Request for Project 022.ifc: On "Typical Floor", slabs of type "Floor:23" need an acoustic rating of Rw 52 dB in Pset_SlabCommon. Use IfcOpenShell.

First a look at what the model holds.

```python
import ifcopenshell
import ifcopenshell.util.element

model = ifcopenshell.open("Project 022.ifc")
print(model.schema)
storey = next(s for s in model.by_type("IfcBuildingStorey") if s.Name == "Typical Floor")
slabs = [e for e in ifcopenshell.util.element.get_decomposition(storey) if e.is_a("IfcSlab")]
seen = {}
for e in slabs:
    element_type = ifcopenshell.util.element.get_type(e)
    key = (element_type.Name if element_type != e and element_type else None, ifcopenshell.util.element.get_pset(e, "Pset_SlabCommon", "AcousticRating"))
    seen[key] = seen.get(key, 0) + 1
for (name, value), count in sorted(seen.items(), key=str):
    print(count, "x", name, "|", value)
```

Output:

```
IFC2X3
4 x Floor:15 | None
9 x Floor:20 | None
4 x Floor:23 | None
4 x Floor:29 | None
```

```python
import ifcopenshell
import ifcopenshell.api.pset
import ifcopenshell.util.element

model = ifcopenshell.open("Project 022.ifc")

storey = next(s for s in model.by_type("IfcBuildingStorey") if s.Name == "Typical Floor")
slabs = [e for e in ifcopenshell.util.element.get_decomposition(storey) if e.is_a("IfcSlab")]

count = 0
for e in slabs:
    element_type = ifcopenshell.util.element.get_type(e)
    if element_type in (None, e) or element_type.Name != "Floor:23":
        continue
    # add_pset returns the element's existing set when there is one.
    pset = ifcopenshell.api.pset.add_pset(model, product=e, name="Pset_SlabCommon")
    ifcopenshell.api.pset.edit_pset(model, pset=pset, properties={"AcousticRating": "Rw 52 dB"})
    count += 1

print(count, "slabs updated")

model.write("Project 022-out.ifc")
```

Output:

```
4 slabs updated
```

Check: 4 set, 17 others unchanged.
